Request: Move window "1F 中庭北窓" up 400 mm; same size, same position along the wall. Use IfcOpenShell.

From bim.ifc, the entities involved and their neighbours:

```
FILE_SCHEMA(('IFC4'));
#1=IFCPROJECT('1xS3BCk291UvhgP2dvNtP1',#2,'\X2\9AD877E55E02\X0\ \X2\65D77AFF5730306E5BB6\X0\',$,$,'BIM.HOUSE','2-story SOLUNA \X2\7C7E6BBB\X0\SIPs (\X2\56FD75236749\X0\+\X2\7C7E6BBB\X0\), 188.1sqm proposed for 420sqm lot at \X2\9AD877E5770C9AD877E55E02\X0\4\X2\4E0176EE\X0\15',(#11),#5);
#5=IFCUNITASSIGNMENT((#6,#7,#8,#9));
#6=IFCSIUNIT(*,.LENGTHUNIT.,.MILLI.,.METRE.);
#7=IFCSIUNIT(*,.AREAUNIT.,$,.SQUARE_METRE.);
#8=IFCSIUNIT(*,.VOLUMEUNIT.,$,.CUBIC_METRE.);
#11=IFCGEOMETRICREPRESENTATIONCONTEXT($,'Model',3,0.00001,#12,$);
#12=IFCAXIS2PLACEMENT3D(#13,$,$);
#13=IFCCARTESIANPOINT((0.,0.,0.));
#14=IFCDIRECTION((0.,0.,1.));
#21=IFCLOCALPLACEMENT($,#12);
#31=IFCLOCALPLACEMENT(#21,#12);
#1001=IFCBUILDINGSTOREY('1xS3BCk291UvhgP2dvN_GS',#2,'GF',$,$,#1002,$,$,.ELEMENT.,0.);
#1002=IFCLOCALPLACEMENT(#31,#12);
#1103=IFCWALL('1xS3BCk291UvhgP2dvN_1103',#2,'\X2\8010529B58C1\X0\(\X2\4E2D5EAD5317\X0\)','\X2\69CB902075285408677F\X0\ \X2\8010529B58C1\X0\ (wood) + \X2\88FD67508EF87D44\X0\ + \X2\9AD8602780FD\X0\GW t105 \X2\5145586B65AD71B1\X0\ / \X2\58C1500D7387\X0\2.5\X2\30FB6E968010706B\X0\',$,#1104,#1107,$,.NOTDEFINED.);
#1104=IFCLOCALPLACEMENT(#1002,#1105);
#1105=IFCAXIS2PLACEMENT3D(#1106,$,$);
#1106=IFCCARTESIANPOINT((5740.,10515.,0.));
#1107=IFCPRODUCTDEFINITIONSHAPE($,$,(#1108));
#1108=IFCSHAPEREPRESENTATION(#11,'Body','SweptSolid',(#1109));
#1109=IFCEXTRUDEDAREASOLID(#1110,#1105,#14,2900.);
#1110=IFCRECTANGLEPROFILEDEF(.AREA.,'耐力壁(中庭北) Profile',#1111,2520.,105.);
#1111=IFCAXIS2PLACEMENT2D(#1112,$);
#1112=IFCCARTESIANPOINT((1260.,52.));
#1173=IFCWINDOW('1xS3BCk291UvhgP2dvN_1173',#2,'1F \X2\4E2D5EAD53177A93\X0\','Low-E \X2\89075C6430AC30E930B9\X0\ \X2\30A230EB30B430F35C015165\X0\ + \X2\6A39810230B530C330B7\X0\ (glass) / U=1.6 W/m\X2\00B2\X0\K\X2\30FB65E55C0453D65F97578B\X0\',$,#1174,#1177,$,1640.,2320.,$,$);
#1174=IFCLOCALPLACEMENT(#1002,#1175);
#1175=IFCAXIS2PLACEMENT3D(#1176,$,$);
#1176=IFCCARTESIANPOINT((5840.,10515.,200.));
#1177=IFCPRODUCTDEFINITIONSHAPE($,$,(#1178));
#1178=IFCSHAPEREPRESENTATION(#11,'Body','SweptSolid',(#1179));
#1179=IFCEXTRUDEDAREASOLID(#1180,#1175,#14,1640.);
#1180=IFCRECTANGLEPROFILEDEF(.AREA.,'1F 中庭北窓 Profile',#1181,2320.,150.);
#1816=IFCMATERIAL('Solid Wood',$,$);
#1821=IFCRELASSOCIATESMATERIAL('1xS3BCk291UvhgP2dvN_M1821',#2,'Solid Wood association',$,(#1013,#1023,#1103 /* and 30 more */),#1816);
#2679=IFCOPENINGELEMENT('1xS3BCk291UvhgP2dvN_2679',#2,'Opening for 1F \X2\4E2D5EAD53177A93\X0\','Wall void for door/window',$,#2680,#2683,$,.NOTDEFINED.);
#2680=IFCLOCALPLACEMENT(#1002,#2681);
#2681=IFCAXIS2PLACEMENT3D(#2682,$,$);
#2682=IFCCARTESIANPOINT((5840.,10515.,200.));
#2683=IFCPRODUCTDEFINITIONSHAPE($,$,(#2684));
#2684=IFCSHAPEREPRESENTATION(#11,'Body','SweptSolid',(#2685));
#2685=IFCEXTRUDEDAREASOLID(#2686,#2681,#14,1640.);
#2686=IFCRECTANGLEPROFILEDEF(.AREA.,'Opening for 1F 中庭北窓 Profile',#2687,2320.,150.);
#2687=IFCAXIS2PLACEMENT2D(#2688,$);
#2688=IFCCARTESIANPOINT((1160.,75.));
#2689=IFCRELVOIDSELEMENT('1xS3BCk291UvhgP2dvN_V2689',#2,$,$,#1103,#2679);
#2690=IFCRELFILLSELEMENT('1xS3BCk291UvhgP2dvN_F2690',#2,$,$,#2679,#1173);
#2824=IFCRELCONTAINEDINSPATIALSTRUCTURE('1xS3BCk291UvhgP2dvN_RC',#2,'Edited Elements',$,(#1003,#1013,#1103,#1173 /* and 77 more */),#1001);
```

```python
import numpy as np
import ifcopenshell
import ifcopenshell.api.geometry
import ifcopenshell.util.placement
import ifcopenshell.util.unit

model = ifcopenshell.open("bim.ifc")
unit_scale = ifcopenshell.util.unit.calculate_unit_scale(model)

window = model.by_id(1173)
opening = window.FillsVoids[0].RelatingOpeningElement
dz = 0.4 / unit_scale

shift = np.array([0.0, 0.0, dz])
# The window is not placed relative to its opening, so move both.
for product in (opening, window):
    matrix = ifcopenshell.util.placement.get_local_placement(product.ObjectPlacement)
    matrix[:3, 3] += shift
    ifcopenshell.api.geometry.edit_object_placement(model, product=product, matrix=matrix, is_si=False)

print(f"moved by {dz * unit_scale:+.3f} m")

model.write("bim-out.ifc")
```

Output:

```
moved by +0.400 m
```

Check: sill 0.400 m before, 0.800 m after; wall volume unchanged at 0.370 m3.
